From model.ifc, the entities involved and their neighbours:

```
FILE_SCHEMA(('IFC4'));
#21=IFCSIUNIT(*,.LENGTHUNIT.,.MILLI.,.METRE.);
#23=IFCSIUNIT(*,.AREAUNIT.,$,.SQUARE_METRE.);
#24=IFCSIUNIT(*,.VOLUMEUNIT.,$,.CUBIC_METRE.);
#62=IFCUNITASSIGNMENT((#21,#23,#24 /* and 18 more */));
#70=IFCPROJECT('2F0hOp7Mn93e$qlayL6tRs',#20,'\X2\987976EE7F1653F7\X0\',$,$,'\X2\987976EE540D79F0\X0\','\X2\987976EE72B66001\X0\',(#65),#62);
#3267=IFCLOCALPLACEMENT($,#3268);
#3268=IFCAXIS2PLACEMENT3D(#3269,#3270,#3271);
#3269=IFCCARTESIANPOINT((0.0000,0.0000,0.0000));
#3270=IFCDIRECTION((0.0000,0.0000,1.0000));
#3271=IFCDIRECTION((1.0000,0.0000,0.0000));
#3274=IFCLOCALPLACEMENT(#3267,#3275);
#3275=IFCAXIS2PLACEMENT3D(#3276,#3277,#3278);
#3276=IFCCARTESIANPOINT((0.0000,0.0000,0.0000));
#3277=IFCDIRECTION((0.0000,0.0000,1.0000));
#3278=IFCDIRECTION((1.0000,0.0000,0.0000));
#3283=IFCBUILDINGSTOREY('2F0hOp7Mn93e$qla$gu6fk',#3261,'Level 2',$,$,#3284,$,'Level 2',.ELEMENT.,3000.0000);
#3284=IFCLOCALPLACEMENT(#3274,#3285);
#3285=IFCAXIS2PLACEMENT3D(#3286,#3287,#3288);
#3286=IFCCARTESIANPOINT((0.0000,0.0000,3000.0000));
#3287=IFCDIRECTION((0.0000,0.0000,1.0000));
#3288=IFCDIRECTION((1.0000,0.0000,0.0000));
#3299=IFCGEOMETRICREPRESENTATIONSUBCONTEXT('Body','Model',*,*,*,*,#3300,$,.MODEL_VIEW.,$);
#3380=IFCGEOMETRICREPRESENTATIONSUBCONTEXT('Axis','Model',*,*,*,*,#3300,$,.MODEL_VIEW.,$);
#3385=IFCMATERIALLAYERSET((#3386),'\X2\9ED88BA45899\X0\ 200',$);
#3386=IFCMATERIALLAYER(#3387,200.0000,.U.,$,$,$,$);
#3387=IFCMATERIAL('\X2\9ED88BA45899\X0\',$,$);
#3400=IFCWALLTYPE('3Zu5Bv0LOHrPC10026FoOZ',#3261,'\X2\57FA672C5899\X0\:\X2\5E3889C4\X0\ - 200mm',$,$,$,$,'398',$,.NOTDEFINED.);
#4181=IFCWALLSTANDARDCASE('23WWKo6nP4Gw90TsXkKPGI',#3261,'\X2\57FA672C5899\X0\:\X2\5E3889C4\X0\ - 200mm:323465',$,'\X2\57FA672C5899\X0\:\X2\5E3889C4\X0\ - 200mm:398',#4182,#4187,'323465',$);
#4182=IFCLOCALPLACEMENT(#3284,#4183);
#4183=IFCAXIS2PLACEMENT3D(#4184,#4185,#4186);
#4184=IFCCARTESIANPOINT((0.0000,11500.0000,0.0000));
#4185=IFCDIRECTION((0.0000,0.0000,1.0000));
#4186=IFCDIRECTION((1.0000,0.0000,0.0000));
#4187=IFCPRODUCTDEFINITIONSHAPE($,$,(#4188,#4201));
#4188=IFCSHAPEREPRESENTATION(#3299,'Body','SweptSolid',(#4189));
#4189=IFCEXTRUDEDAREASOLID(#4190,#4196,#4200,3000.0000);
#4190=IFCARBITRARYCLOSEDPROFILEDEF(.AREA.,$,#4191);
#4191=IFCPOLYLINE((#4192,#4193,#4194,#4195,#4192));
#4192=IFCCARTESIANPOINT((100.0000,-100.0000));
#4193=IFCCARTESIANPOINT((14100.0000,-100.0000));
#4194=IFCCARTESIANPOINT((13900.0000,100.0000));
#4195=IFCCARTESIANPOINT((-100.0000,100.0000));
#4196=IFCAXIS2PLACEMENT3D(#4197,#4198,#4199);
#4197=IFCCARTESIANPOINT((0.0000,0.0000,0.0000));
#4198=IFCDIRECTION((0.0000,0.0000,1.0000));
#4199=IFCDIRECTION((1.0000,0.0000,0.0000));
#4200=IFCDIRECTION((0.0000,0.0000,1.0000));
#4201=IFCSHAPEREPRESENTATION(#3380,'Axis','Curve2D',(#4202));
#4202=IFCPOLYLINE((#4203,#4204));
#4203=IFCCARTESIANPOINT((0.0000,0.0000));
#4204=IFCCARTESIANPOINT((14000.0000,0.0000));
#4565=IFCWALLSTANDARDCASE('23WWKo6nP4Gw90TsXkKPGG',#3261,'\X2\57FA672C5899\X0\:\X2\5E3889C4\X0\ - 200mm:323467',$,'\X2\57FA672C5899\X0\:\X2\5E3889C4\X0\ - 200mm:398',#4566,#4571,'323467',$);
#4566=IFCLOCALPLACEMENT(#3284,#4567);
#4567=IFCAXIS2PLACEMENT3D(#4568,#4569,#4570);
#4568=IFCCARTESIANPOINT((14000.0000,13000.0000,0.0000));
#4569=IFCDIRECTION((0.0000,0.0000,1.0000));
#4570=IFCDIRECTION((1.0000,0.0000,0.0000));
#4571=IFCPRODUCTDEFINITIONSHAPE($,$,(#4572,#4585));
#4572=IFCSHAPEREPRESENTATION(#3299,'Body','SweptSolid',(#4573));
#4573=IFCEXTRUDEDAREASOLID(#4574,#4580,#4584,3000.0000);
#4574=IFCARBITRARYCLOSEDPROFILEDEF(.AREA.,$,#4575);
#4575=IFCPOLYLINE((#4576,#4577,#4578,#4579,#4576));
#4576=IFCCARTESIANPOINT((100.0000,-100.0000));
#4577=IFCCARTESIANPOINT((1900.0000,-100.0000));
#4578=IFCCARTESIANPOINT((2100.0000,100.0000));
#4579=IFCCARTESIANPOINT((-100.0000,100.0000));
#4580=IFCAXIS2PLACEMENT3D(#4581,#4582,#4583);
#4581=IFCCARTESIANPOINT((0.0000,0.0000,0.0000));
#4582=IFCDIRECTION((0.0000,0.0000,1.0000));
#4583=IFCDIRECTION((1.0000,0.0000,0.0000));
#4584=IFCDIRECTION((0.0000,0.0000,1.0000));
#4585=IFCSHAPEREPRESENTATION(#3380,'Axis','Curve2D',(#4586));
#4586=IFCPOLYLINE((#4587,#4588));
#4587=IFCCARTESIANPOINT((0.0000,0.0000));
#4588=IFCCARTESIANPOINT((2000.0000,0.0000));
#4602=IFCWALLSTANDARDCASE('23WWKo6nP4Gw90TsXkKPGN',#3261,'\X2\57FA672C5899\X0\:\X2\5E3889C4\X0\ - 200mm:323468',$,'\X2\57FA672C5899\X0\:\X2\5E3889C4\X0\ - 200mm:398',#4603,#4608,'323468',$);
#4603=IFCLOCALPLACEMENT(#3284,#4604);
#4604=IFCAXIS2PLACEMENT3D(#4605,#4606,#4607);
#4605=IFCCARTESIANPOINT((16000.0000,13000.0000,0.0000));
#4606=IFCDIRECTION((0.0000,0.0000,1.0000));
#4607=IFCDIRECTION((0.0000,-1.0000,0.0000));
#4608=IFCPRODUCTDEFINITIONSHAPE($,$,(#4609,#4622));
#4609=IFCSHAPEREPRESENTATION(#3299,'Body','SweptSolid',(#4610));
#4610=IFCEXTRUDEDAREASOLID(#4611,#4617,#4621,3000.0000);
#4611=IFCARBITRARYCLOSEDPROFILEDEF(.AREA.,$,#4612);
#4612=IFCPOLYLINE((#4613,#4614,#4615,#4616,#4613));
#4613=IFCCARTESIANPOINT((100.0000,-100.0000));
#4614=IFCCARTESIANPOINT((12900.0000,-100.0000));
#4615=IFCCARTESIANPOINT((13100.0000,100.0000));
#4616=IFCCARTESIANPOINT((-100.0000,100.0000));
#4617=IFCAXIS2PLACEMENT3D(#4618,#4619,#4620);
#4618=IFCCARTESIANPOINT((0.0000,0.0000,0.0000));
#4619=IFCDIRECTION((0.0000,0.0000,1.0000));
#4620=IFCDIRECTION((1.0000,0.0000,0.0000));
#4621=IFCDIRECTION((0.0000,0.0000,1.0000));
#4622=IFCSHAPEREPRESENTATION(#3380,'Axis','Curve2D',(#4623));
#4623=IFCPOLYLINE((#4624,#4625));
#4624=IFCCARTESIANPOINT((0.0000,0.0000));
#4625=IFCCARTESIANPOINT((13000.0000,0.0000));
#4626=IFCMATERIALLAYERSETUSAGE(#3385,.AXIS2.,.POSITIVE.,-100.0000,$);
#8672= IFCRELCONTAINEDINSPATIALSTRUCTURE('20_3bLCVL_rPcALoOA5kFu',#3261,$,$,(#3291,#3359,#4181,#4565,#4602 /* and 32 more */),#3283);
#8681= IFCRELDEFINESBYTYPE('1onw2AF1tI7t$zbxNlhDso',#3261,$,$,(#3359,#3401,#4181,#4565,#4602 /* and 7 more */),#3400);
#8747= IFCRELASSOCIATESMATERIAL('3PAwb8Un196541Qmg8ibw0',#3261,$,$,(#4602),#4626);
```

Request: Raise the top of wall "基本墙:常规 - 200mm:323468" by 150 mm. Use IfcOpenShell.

```python
import ifcopenshell
import ifcopenshell.geom
import ifcopenshell.util.representation
import ifcopenshell.util.shape

model = ifcopenshell.open("model.ifc")
settings = ifcopenshell.geom.settings()


def volume(element):
    """Net volume in cubic metres, openings subtracted."""
    shape = ifcopenshell.geom.create_shape(settings, element)
    return ifcopenshell.util.shape.get_volume(shape.geometry)


wall = model.by_guid("23WWKo6nP4Gw90TsXkKPGN")
before = volume(wall)

body = ifcopenshell.util.representation.get_representation(wall, "Model", "Body")
solid = body.Items[0]
old_height = solid.Depth
solid.Depth += 150.0
after = volume(wall)

print(f"height {old_height:g} -> {solid.Depth:g}, volume {before:.3f} -> {after:.3f} m3")

model.write("model_rev.ifc")
```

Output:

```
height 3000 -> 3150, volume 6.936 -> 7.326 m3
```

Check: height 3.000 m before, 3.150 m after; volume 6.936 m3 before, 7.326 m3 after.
